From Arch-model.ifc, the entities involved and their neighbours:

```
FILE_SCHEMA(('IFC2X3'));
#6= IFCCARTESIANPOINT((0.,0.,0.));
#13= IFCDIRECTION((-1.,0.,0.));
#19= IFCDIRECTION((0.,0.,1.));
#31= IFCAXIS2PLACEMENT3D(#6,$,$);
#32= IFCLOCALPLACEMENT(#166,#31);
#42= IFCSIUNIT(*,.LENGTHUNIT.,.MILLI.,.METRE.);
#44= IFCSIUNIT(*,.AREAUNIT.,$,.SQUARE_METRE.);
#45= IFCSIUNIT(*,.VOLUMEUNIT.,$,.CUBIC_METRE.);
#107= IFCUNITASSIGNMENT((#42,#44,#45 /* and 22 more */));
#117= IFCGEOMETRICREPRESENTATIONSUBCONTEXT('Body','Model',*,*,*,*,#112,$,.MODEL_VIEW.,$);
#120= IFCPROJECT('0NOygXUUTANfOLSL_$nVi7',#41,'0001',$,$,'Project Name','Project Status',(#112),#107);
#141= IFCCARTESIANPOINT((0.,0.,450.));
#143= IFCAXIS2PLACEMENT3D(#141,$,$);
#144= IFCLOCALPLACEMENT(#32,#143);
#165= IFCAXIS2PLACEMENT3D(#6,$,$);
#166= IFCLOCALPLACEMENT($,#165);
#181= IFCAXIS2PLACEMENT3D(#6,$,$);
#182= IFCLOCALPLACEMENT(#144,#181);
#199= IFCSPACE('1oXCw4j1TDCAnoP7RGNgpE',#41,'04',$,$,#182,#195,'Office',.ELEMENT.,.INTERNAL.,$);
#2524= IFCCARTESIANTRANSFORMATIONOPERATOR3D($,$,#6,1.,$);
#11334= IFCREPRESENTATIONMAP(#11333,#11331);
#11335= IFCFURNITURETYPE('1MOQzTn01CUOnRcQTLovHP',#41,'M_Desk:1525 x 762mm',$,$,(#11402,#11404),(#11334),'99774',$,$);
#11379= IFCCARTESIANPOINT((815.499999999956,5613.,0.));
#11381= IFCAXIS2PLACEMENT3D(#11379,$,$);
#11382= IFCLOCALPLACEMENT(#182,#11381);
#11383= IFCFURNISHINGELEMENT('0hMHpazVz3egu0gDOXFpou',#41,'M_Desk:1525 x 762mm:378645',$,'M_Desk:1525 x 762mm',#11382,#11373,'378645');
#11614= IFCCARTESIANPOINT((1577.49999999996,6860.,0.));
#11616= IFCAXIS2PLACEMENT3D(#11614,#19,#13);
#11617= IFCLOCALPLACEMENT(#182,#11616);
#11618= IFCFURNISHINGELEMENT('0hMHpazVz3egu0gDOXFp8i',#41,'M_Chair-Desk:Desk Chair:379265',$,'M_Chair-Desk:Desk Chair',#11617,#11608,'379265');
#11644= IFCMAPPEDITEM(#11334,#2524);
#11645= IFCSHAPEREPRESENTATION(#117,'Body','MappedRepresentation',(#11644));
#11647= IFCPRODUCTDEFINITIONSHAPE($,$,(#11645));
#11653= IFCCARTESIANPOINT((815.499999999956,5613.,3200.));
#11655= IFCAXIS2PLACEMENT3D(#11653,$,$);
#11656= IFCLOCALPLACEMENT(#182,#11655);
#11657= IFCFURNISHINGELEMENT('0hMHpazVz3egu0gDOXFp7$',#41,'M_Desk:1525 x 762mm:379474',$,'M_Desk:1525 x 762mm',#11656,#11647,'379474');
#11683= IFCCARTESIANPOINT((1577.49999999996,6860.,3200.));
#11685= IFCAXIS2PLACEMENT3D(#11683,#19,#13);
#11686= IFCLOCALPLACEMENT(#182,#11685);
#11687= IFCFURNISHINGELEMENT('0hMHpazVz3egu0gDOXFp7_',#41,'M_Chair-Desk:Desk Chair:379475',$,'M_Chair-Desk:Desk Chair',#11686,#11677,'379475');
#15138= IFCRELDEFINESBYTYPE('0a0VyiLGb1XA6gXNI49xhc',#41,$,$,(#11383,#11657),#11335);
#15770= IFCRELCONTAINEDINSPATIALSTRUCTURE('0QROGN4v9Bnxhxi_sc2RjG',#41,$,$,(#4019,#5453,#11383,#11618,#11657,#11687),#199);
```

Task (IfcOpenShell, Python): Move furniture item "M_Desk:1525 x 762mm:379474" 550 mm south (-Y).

```python
import ifcopenshell
import ifcopenshell.api.geometry
import ifcopenshell.util.placement
import ifcopenshell.util.unit

model = ifcopenshell.open("Arch-model.ifc")
unit_scale = ifcopenshell.util.unit.calculate_unit_scale(model)

item = model.by_guid("0hMHpazVz3egu0gDOXFp7$")
matrix = ifcopenshell.util.placement.get_local_placement(item.ObjectPlacement)
matrix[1, 3] -= 0.55 / unit_scale
ifcopenshell.api.geometry.edit_object_placement(model, product=item, matrix=matrix, is_si=False)

print(ifcopenshell.util.placement.get_local_placement(item.ObjectPlacement).round(3) + 0.0)

model.write("Arch-model_updated.ifc")
```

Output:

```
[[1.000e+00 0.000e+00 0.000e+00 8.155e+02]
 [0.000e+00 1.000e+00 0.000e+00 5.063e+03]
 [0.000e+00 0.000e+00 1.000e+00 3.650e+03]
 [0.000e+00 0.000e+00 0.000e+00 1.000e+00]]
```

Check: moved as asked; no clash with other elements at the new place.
